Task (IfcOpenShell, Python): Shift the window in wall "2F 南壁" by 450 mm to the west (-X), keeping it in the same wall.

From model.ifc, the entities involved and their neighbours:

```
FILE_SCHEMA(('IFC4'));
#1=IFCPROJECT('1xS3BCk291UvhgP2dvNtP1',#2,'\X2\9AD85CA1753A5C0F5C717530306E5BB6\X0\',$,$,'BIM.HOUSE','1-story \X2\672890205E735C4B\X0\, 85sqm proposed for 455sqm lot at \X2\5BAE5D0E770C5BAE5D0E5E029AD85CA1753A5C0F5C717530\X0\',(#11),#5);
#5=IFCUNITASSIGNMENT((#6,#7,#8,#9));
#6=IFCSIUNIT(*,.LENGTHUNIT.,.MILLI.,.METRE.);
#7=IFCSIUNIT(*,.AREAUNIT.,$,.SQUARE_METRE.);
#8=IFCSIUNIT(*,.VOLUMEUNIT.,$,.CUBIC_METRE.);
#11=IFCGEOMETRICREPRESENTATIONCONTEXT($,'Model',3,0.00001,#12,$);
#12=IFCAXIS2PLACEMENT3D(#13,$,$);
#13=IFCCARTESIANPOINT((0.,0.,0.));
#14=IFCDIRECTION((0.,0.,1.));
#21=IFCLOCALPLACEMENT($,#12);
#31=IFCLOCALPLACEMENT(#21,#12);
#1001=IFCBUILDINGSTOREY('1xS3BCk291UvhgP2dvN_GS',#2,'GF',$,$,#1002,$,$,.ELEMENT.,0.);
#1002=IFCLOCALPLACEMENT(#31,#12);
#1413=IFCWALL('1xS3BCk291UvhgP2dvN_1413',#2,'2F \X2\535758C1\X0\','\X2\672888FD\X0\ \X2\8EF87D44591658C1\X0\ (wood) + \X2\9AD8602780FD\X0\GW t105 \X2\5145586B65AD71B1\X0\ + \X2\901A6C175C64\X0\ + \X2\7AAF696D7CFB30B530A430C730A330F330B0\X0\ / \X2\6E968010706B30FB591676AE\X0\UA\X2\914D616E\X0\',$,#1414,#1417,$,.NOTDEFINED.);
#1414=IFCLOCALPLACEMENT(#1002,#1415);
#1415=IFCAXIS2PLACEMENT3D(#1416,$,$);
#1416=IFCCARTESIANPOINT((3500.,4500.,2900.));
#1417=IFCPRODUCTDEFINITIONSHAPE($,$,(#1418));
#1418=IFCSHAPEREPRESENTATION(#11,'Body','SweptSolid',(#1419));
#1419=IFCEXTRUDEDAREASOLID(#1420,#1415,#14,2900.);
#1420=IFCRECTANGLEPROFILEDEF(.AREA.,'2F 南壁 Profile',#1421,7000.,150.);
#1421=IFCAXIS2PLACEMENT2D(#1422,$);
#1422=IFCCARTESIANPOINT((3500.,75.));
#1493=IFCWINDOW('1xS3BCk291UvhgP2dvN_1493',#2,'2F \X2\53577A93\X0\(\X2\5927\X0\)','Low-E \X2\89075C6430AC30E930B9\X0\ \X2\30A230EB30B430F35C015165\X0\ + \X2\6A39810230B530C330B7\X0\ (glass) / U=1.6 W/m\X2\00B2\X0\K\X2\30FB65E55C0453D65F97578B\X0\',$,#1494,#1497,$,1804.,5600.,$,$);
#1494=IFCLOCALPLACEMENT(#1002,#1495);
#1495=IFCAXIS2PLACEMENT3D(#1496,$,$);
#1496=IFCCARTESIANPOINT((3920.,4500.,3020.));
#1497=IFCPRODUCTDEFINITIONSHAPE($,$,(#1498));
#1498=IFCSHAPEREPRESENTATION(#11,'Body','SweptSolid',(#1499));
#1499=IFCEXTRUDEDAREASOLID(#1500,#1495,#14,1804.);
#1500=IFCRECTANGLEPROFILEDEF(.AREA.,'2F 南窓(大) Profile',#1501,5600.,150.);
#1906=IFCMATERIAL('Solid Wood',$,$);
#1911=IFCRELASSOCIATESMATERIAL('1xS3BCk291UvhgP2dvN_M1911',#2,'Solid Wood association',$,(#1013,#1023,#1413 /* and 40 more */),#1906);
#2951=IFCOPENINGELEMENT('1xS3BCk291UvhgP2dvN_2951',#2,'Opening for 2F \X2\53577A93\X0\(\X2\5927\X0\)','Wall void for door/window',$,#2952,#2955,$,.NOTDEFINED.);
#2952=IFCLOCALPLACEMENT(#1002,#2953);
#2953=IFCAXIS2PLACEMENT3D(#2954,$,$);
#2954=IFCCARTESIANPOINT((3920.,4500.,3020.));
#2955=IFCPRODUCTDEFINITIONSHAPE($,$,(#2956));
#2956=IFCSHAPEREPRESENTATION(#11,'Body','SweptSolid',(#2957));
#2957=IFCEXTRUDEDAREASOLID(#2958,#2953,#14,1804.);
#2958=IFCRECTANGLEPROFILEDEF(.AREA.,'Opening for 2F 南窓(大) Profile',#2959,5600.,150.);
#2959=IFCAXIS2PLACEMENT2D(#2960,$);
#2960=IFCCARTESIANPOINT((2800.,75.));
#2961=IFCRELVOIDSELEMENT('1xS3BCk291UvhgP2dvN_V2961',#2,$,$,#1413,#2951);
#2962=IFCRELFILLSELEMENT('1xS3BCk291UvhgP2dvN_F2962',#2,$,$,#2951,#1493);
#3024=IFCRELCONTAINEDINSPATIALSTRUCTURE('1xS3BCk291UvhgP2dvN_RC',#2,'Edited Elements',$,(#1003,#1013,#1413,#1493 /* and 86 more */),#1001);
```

```python
import ifcopenshell
import ifcopenshell.api.geometry
import ifcopenshell.util.placement
import ifcopenshell.util.unit

model = ifcopenshell.open("model.ifc")
unit_scale = ifcopenshell.util.unit.calculate_unit_scale(model)

window = model.by_guid("1xS3BCk291UvhgP2dvN_1493")
opening = window.FillsVoids[0].RelatingOpeningElement
wall = opening.VoidsElements[0].RelatingBuildingElement

wall_matrix = ifcopenshell.util.placement.get_local_placement(wall.ObjectPlacement)
shift = wall_matrix[:3, 0] * -0.45 / unit_scale
before = ifcopenshell.util.placement.get_local_placement(window.ObjectPlacement)[:3, 3].copy()

# The window is not placed relative to its opening, so move both.
for product in (opening, window):
    matrix = ifcopenshell.util.placement.get_local_placement(product.ObjectPlacement)
    matrix[:3, 3] += shift
    ifcopenshell.api.geometry.edit_object_placement(model, product=product, matrix=matrix, is_si=False)

after = ifcopenshell.util.placement.get_local_placement(window.ObjectPlacement)[:3, 3]
print("window moved by", (after - before).round(3) + 0.0)

model.write("model_v2.ifc")
```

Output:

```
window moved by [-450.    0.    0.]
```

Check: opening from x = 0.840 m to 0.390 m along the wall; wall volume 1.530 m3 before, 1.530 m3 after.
